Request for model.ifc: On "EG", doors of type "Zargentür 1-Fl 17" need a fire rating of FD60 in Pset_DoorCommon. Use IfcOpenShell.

First a look at what the model holds.

```python
import ifcopenshell
import ifcopenshell.util.element

model = ifcopenshell.open("model.ifc")
print(model.schema)
storey = next(s for s in model.by_type("IfcBuildingStorey") if s.Name == "EG")
doors = [e for e in ifcopenshell.util.element.get_decomposition(storey) if e.is_a("IfcDoor")]
seen = {}
for e in doors:
    element_type = ifcopenshell.util.element.get_type(e)
    key = (element_type.Name if element_type != e and element_type else None, ifcopenshell.util.element.get_pset(e, "Pset_DoorCommon", "FireRating"))
    seen[key] = seen.get(key, 0) + 1
for (name, value), count in sorted(seen.items(), key=str):
    print(count, "x", name, "|", value)
```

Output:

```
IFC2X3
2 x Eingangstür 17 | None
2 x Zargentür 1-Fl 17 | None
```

```python
import ifcopenshell
import ifcopenshell.api.pset
import ifcopenshell.util.element

model = ifcopenshell.open("model.ifc")

storey = next(s for s in model.by_type("IfcBuildingStorey") if s.Name == "EG")
doors = [e for e in ifcopenshell.util.element.get_decomposition(storey) if e.is_a("IfcDoor")]

count = 0
for e in doors:
    element_type = ifcopenshell.util.element.get_type(e)
    if element_type in (None, e) or element_type.Name != "Zargentür 1-Fl 17":
        continue
    # add_pset returns the element's existing set when there is one.
    pset = ifcopenshell.api.pset.add_pset(model, product=e, name="Pset_DoorCommon")
    ifcopenshell.api.pset.edit_pset(model, pset=pset, properties={"FireRating": "FD60"})
    count += 1

print(count, "doors updated")

model.write("model-out.ifc")
```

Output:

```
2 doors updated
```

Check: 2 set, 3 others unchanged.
